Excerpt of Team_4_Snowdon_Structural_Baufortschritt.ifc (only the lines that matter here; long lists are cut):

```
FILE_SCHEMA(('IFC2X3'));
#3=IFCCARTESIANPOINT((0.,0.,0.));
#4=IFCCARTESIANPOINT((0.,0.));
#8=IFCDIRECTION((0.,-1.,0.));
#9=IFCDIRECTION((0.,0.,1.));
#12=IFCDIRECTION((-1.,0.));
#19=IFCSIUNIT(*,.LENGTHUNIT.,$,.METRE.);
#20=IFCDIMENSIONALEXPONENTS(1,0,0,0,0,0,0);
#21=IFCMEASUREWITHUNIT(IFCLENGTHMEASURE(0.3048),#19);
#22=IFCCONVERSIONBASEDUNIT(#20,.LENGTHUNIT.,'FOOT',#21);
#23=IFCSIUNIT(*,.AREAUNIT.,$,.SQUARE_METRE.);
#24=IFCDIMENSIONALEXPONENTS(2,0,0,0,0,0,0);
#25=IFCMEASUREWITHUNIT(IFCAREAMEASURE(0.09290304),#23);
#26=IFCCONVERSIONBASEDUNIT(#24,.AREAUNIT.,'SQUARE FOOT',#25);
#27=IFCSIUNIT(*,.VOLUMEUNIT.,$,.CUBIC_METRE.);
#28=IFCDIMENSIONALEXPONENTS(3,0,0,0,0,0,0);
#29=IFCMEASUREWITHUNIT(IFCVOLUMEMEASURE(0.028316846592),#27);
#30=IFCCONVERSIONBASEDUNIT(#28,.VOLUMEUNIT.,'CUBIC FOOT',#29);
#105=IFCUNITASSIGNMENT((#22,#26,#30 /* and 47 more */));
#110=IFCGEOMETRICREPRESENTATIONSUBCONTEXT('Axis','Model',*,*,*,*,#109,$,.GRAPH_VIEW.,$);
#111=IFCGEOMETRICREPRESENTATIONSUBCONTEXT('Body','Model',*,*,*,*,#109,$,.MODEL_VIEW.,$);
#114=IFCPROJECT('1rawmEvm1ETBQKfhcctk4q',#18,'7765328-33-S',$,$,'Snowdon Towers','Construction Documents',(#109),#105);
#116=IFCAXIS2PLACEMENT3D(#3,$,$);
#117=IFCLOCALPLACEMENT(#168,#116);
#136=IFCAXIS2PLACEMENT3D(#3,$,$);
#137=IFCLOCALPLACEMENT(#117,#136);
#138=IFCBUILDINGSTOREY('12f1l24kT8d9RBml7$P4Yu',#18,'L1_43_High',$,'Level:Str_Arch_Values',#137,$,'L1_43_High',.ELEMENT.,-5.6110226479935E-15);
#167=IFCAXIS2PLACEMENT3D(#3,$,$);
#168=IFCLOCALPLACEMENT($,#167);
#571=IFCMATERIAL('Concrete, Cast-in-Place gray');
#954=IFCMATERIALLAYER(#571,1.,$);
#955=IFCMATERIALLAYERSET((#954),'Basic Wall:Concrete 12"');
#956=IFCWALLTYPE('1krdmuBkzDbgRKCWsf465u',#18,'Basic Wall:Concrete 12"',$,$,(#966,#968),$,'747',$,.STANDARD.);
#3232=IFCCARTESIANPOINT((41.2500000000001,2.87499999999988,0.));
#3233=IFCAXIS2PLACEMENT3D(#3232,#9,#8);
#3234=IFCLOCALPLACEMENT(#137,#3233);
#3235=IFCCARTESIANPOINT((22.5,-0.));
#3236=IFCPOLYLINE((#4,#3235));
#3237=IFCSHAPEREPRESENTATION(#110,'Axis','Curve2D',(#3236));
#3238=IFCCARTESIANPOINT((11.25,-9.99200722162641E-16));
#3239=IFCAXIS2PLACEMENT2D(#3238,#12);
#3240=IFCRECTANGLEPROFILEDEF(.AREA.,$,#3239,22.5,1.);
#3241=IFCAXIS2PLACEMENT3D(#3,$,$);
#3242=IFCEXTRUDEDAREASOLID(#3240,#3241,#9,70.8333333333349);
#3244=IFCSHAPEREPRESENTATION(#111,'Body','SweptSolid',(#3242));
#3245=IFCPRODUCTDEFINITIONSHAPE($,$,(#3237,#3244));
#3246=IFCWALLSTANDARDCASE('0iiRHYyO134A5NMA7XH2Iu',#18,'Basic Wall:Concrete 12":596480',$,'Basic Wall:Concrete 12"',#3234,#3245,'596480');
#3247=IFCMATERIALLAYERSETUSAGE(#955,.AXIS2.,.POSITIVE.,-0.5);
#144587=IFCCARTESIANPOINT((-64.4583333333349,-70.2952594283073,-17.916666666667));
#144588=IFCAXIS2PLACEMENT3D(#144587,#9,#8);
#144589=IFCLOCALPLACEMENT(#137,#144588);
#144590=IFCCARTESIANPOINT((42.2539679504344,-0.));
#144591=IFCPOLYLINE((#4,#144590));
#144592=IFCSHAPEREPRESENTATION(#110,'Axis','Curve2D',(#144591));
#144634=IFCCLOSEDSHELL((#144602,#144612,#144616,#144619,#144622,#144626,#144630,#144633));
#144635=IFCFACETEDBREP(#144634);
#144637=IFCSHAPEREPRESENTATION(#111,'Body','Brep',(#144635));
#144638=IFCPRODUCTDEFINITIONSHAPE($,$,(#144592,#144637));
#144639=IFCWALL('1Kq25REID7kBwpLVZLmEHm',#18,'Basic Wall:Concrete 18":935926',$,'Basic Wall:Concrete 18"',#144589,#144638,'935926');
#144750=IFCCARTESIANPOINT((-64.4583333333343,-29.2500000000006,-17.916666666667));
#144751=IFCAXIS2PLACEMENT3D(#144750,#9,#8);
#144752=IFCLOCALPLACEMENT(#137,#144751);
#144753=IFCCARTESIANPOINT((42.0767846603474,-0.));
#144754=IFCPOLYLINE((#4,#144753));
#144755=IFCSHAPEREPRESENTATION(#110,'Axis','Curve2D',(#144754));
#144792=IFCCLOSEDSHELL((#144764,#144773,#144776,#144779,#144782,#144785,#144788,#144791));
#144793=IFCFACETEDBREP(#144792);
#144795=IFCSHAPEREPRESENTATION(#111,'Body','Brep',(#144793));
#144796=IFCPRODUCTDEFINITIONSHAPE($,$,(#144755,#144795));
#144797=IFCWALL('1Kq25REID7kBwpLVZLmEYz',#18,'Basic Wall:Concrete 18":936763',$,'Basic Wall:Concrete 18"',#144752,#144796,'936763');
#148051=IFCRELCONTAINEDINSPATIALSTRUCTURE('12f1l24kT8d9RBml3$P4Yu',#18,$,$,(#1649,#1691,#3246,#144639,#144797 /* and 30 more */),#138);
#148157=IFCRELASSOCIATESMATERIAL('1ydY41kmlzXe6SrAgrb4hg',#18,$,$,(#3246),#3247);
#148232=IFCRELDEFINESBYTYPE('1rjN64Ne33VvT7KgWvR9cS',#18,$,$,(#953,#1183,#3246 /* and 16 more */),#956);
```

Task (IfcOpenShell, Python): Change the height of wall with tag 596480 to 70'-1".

```python
import ifcopenshell
import ifcopenshell.geom
import ifcopenshell.util.representation
import ifcopenshell.util.shape
import ifcopenshell.util.unit

model = ifcopenshell.open("Team_4_Snowdon_Structural_Baufortschritt.ifc")
unit_scale = ifcopenshell.util.unit.calculate_unit_scale(model)
settings = ifcopenshell.geom.settings()


def volume(element):
    """Net volume in cubic metres, openings subtracted."""
    shape = ifcopenshell.geom.create_shape(settings, element)
    return ifcopenshell.util.shape.get_volume(shape.geometry)


wall = model.by_id(3246)
before = volume(wall)

body = ifcopenshell.util.representation.get_representation(wall, "Model", "Body")
solid = body.Items[0]
old_height = solid.Depth
solid.Depth = 841 * 0.0254 / unit_scale
after = volume(wall)

print(f"height {old_height:g} -> {solid.Depth:g}, volume {before:.3f} -> {after:.3f} m3")

model.write("Team_4_Snowdon_Structural_Baufortschritt_rev.ifc")
```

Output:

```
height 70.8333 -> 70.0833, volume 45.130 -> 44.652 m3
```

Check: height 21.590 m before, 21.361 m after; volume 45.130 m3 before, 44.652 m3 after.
